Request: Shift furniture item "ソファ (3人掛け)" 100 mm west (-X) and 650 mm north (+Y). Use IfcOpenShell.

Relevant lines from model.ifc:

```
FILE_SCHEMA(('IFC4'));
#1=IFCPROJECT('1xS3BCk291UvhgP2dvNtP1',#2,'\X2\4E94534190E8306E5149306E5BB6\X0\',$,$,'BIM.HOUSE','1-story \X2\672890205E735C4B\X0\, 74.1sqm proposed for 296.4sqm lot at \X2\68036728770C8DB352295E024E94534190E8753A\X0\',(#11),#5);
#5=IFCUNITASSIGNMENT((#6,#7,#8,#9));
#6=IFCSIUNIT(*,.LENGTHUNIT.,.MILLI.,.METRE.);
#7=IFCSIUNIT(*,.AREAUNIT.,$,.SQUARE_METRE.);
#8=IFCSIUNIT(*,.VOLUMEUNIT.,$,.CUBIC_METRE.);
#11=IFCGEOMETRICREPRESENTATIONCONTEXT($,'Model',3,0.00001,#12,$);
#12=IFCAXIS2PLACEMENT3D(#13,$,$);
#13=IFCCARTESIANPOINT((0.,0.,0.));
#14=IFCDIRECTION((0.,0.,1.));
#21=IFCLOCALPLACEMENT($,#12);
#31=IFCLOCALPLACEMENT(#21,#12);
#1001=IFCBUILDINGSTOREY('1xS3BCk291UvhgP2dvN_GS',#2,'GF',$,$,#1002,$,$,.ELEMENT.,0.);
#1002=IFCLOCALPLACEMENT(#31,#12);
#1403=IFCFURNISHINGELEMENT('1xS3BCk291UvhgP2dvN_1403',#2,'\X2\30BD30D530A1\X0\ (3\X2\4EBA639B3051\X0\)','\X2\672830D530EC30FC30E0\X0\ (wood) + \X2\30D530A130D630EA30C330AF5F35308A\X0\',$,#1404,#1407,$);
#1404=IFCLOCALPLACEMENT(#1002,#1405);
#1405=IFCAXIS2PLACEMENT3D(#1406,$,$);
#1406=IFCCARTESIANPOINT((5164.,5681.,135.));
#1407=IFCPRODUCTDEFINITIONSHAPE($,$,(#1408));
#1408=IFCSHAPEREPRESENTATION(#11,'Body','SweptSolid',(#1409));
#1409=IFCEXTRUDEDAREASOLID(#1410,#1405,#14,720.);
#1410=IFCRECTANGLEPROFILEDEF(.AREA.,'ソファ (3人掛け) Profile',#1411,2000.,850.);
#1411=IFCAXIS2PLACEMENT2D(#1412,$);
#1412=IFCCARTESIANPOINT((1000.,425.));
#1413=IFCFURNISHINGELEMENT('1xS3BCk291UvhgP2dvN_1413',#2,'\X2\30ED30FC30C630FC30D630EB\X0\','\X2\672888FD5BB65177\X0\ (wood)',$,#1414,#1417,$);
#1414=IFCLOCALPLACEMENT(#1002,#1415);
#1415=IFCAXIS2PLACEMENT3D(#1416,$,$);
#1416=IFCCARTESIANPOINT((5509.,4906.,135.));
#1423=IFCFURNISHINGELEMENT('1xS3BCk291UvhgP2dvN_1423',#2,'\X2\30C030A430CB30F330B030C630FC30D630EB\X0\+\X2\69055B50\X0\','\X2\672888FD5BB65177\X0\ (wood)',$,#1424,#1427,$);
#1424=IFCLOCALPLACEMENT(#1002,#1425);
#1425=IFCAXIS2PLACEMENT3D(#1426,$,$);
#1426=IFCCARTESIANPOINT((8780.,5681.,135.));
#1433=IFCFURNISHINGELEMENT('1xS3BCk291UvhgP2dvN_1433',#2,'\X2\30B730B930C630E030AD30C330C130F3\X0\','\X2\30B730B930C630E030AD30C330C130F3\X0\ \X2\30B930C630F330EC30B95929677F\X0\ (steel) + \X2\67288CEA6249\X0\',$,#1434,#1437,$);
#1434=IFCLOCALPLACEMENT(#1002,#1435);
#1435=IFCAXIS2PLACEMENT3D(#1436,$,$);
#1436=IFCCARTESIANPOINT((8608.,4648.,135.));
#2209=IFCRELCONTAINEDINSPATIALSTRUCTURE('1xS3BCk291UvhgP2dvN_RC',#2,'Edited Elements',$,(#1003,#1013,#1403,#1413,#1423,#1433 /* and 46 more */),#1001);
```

```python
import ifcopenshell
import ifcopenshell.api.geometry
import ifcopenshell.util.placement

model = ifcopenshell.open("model.ifc")

item = model.by_guid("1xS3BCk291UvhgP2dvN_1403")
matrix = ifcopenshell.util.placement.get_local_placement(item.ObjectPlacement)
matrix[0, 3] -= 100.0
matrix[1, 3] += 650.0
ifcopenshell.api.geometry.edit_object_placement(model, product=item, matrix=matrix, is_si=False)

print(ifcopenshell.util.placement.get_local_placement(item.ObjectPlacement).round(3) + 0.0)

model.write("model_v2.ifc")
```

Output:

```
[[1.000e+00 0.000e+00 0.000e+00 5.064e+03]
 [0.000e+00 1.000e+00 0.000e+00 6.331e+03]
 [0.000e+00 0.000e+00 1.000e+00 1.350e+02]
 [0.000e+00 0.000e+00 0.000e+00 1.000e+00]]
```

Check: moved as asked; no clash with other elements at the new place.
